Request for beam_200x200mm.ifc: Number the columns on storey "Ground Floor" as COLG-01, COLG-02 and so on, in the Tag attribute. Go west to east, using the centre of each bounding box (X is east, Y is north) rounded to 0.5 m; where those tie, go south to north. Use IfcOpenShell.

First a look at what the model holds.

```python
import ifcopenshell
import ifcopenshell.util.element
import ifcopenshell.util.placement

model = ifcopenshell.open("beam_200x200mm.ifc")
print(model.schema)
storey = next(s for s in model.by_type("IfcBuildingStorey") if s.Name == "Ground Floor")
columns = [e for e in ifcopenshell.util.element.get_decomposition(storey) if e.is_a("IfcColumn")]
for e in sorted(columns, key=lambda e: e.id()):
    origin = ifcopenshell.util.placement.get_local_placement(e.ObjectPlacement)[:3, 3]
    print(e.id(), e.Tag, e.Name, origin.round(2) + 0.0, sep=" | ")
```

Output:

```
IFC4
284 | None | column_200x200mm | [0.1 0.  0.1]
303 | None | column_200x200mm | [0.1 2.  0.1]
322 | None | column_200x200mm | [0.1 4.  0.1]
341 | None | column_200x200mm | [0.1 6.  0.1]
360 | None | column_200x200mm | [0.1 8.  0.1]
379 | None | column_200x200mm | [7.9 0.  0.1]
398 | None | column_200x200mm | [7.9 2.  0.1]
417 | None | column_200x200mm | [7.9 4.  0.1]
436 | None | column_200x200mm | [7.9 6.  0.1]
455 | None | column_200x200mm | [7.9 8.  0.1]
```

```python
import ifcopenshell
import ifcopenshell.geom
import ifcopenshell.util.element
import ifcopenshell.util.shape

model = ifcopenshell.open("beam_200x200mm.ifc")
settings = ifcopenshell.geom.settings()
settings.set("use-world-coords", True)


def centre(element):
    shape = ifcopenshell.geom.create_shape(settings, element)
    return ifcopenshell.util.shape.get_bbox_centroid(shape.geometry)


storey = next(s for s in model.by_type("IfcBuildingStorey") if s.Name == "Ground Floor")
columns = [e for e in ifcopenshell.util.element.get_decomposition(storey) if e.is_a("IfcColumn")]

# Insertion points can sit at a corner or the storey origin, so sort by the geometry (in metres).
centres = {e: centre(e) for e in columns}
columns.sort(key=lambda e: (round(centres[e][0] / 0.5), centres[e][1]))

for i, e in enumerate(columns, start=1):
    number = f"COLG-{i:02d}"
    e.Tag = number
    print(e.id(), number)

model.write("beam_200x200mm-out.ifc")
```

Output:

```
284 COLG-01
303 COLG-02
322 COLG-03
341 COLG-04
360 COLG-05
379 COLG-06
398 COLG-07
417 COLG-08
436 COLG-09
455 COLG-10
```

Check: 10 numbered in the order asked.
